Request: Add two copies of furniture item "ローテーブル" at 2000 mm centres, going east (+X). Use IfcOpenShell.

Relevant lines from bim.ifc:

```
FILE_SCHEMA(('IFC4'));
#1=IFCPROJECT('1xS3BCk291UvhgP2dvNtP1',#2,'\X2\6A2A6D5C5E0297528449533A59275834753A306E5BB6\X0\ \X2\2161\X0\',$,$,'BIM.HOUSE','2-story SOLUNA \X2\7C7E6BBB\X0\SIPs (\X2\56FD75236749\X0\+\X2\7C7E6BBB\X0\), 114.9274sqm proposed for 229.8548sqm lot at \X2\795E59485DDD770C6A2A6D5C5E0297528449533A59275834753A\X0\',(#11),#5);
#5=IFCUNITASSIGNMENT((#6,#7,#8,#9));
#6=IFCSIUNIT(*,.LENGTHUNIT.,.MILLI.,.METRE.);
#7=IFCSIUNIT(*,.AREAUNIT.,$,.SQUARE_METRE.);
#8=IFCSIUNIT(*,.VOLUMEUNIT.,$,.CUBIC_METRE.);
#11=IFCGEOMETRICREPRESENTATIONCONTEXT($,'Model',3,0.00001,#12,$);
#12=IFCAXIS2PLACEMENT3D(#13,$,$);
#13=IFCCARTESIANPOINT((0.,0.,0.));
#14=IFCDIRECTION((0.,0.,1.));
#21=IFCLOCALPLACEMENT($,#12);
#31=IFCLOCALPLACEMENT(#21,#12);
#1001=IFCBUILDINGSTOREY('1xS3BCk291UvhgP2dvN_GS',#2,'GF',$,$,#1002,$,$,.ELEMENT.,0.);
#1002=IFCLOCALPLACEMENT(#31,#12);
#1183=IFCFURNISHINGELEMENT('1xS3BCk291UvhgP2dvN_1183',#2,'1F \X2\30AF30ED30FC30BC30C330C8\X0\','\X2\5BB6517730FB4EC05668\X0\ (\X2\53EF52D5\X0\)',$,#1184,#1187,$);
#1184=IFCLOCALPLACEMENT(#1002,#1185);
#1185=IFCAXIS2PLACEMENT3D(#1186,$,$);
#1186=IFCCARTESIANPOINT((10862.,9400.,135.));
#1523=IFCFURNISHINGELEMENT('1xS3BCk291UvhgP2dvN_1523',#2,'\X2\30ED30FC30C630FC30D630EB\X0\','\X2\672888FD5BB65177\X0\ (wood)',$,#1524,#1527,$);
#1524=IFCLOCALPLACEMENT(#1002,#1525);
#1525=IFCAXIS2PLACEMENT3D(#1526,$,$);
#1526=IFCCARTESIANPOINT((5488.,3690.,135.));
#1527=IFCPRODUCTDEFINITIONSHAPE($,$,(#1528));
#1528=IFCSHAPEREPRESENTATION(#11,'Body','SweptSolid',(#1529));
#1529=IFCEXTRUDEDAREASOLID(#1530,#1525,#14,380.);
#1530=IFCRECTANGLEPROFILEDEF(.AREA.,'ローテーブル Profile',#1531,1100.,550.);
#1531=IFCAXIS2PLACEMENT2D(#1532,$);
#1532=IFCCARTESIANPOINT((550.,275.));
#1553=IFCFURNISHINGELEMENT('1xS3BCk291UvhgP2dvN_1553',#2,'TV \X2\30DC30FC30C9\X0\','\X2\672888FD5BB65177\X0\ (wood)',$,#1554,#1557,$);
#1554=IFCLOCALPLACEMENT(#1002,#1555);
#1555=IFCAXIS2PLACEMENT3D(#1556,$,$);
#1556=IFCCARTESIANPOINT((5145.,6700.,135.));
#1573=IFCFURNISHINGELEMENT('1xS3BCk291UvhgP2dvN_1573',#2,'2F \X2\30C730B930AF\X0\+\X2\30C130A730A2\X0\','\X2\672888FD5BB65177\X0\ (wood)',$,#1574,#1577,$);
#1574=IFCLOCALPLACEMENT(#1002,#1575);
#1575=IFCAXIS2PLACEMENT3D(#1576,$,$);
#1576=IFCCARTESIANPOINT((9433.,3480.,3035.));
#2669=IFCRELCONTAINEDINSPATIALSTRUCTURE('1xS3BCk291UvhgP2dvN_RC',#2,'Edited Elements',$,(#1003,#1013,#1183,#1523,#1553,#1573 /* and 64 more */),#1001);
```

```python
import numpy as np
import ifcopenshell
import ifcopenshell.api.geometry
import ifcopenshell.api.root
import ifcopenshell.util.element
import ifcopenshell.util.placement
import ifcopenshell.util.unit

model = ifcopenshell.open("bim.ifc")
unit_scale = ifcopenshell.util.unit.calculate_unit_scale(model)


def reuse_history(source, copy):
    """copy_class also copies each property set's owner history, people and application; keep the originals."""
    for rel in copy.IsDefinedBy:
        if rel.is_a("IfcRelDefinesByProperties") and (history := rel.RelatingPropertyDefinition.OwnerHistory):
            rel.RelatingPropertyDefinition.OwnerHistory = source.OwnerHistory
            ifcopenshell.util.element.remove_deep2(model, history)


source = model.by_id(1523)
base = ifcopenshell.util.placement.get_local_placement(source.ObjectPlacement)
step = np.array([1.0, 0.0, 0.0]) * 2 / unit_scale

for i in range(1, 3):
    copy = ifcopenshell.api.root.copy_class(model, product=source)
    copy.Representation = ifcopenshell.util.element.copy_deep(
        model, source.Representation, exclude=["IfcGeometricRepresentationContext", "IfcRepresentationMap"]
    )
    reuse_history(source, copy)
    matrix = base.copy()
    matrix[:3, 3] += i * step
    print("added at", matrix[:3, 3].round(3) + 0.0)
    ifcopenshell.api.geometry.edit_object_placement(model, product=copy, matrix=matrix, is_si=False)

model.write("bim_edited.ifc")
```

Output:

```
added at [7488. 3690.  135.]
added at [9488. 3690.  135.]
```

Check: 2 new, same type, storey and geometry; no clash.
